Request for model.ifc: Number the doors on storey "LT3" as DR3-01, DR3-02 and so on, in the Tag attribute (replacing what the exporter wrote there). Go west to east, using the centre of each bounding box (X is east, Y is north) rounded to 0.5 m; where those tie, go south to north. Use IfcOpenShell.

First a look at what the model holds.

```python
import ifcopenshell
import ifcopenshell.util.element
import ifcopenshell.util.placement

model = ifcopenshell.open("model.ifc")
print(model.schema)
storey = next(s for s in model.by_type("IfcBuildingStorey") if s.Name == "LT3")
doors = [e for e in ifcopenshell.util.element.get_decomposition(storey) if e.is_a("IfcDoor")]
for e in sorted(doors, key=lambda e: e.id()):
    origin = ifcopenshell.util.placement.get_local_placement(e.ObjectPlacement)[:3, 3]
    print(e.id(), e.Tag, e.Name, origin.round(2) + 0.0, sep=" | ")
```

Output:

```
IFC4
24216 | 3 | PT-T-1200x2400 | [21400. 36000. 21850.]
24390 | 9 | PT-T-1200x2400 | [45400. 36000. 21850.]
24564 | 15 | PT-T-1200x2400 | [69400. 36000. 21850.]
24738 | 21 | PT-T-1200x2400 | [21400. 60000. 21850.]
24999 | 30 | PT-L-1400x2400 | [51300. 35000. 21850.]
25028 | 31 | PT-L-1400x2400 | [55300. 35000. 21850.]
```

```python
import ifcopenshell
import ifcopenshell.geom
import ifcopenshell.util.element
import ifcopenshell.util.shape

model = ifcopenshell.open("model.ifc")
settings = ifcopenshell.geom.settings()
settings.set("use-world-coords", True)


def centre(element):
    shape = ifcopenshell.geom.create_shape(settings, element)
    return ifcopenshell.util.shape.get_bbox_centroid(shape.geometry)


storey = next(s for s in model.by_type("IfcBuildingStorey") if s.Name == "LT3")
doors = [e for e in ifcopenshell.util.element.get_decomposition(storey) if e.is_a("IfcDoor")]

# Insertion points can sit at a corner or the storey origin, so sort by the geometry (in metres).
centres = {e: centre(e) for e in doors}
doors.sort(key=lambda e: (round(centres[e][0] / 0.5), centres[e][1]))

for i, e in enumerate(doors, start=1):
    number = f"DR3-{i:02d}"
    e.Tag = number
    print(e.id(), number)

model.write("model_edited.ifc")
```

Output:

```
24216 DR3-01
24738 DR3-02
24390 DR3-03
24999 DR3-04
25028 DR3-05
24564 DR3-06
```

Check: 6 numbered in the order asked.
